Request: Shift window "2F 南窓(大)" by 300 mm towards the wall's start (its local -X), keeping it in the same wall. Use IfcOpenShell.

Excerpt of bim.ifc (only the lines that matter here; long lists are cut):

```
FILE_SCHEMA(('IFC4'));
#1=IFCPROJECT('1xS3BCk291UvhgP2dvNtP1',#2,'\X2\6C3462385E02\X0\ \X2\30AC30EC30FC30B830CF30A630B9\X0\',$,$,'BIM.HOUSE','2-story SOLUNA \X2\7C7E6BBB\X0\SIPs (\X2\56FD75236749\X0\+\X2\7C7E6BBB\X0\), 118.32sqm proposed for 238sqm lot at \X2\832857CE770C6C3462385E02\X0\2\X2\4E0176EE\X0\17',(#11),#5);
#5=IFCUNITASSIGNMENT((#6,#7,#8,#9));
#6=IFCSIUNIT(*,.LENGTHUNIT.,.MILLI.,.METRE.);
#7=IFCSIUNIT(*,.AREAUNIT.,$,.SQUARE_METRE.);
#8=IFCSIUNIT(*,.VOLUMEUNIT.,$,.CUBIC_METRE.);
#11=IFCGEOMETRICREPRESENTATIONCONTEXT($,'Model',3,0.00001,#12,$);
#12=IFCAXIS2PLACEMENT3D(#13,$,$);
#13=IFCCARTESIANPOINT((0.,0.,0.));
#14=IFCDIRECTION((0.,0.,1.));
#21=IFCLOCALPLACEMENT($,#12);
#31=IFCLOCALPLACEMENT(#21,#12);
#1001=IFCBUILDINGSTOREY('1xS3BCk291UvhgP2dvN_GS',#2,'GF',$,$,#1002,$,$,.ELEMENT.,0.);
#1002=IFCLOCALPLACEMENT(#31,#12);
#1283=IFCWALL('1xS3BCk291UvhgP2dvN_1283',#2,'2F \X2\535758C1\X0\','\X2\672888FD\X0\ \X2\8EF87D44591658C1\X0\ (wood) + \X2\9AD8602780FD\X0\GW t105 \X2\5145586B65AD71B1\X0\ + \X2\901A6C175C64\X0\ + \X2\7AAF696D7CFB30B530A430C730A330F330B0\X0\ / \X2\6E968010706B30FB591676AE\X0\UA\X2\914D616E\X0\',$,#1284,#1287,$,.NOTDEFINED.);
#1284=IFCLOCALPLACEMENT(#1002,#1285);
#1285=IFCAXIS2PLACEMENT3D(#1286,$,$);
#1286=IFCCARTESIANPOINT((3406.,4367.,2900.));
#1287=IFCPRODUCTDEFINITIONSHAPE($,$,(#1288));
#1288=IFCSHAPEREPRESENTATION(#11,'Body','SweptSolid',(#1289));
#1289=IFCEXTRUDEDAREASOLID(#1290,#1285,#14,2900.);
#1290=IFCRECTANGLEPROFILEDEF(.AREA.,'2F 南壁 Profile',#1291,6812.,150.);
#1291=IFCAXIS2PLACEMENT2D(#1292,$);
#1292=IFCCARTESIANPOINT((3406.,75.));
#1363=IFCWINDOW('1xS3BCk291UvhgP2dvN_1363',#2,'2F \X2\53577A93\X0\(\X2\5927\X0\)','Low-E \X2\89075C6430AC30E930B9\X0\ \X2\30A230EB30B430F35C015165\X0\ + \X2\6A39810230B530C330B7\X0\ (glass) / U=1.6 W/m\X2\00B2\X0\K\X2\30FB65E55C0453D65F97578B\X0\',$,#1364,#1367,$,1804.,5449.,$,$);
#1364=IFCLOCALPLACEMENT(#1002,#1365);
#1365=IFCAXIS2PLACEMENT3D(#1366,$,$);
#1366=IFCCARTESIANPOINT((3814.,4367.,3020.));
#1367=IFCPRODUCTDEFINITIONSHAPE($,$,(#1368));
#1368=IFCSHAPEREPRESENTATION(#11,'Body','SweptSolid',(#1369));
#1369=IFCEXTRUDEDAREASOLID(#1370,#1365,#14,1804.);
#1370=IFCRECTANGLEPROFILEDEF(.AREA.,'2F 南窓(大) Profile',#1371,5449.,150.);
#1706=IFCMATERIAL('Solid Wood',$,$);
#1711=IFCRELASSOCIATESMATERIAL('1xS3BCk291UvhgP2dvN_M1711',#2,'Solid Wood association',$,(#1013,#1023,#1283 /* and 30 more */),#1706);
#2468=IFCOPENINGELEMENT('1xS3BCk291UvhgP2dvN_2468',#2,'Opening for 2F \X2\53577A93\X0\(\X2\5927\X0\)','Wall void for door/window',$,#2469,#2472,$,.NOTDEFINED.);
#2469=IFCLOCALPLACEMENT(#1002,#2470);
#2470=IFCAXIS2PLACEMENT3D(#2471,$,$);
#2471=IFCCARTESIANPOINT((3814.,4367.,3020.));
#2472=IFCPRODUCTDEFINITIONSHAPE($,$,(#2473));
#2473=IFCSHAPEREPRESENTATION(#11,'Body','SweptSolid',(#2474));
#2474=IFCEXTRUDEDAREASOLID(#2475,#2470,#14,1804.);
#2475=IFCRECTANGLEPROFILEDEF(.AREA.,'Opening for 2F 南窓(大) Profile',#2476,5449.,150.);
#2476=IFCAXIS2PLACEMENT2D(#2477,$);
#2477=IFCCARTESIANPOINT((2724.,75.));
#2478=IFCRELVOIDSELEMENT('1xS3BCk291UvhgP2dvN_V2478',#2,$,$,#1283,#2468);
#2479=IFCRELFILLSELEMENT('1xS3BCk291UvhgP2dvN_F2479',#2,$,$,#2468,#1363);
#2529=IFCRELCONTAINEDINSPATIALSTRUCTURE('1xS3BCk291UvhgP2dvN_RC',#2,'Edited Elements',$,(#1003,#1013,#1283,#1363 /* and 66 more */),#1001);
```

```python
import ifcopenshell
import ifcopenshell.api.geometry
import ifcopenshell.util.placement
import ifcopenshell.util.unit

model = ifcopenshell.open("bim.ifc")
unit_scale = ifcopenshell.util.unit.calculate_unit_scale(model)

window = model.by_guid("1xS3BCk291UvhgP2dvN_1363")
opening = window.FillsVoids[0].RelatingOpeningElement
wall = opening.VoidsElements[0].RelatingBuildingElement

wall_matrix = ifcopenshell.util.placement.get_local_placement(wall.ObjectPlacement)
shift = wall_matrix[:3, 0] * -0.3 / unit_scale
before = ifcopenshell.util.placement.get_local_placement(window.ObjectPlacement)[:3, 3].copy()

# The window is not placed relative to its opening, so move both.
for product in (opening, window):
    matrix = ifcopenshell.util.placement.get_local_placement(product.ObjectPlacement)
    matrix[:3, 3] += shift
    ifcopenshell.api.geometry.edit_object_placement(model, product=product, matrix=matrix, is_si=False)

after = ifcopenshell.util.placement.get_local_placement(window.ObjectPlacement)[:3, 3]
print("window moved by", (after - before).round(3) + 0.0)

model.write("bim_v2.ifc")
```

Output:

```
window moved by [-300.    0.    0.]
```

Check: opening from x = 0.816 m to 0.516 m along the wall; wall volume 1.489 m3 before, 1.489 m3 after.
